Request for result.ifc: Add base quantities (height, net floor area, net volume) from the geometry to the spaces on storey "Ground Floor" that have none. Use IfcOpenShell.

First a look at what the model holds.

```python
import ifcopenshell
import ifcopenshell.util.element
import ifcopenshell.util.unit

model = ifcopenshell.open("result.ifc")
print(model.schema)
for unit_type in ("LENGTHUNIT", "AREAUNIT", "VOLUMEUNIT"):
    print(unit_type, ifcopenshell.util.unit.calculate_unit_scale(model, unit_type))
storey = next(s for s in model.by_type("IfcBuildingStorey") if s.Name == "Ground Floor")
spaces = [e for e in ifcopenshell.util.element.get_decomposition(storey) if e.is_a("IfcSpace")]
for e in sorted(spaces, key=lambda e: e.id()):
    print(e.id(), e.is_a(), e.Name, list(ifcopenshell.util.element.get_psets(e, qtos_only=True)), sep=" | ")
```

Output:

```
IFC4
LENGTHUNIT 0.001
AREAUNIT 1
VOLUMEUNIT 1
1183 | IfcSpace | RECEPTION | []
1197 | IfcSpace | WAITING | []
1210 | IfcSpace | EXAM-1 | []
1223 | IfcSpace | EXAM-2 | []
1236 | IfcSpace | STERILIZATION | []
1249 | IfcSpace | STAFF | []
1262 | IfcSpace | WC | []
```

```python
import ifcopenshell
import ifcopenshell.api.pset
import ifcopenshell.geom
import ifcopenshell.util.element
import ifcopenshell.util.shape
import ifcopenshell.util.unit

model = ifcopenshell.open("result.ifc")
unit_scale = ifcopenshell.util.unit.calculate_unit_scale(model)
area_scale = ifcopenshell.util.unit.calculate_unit_scale(model, "AREAUNIT")
volume_scale = ifcopenshell.util.unit.calculate_unit_scale(model, "VOLUMEUNIT")
settings = ifcopenshell.geom.settings()

storey = next(s for s in model.by_type("IfcBuildingStorey") if s.Name == "Ground Floor")
spaces = [e for e in ifcopenshell.util.element.get_decomposition(storey) if e.is_a("IfcSpace")]

for e in sorted(spaces, key=lambda e: e.id()):
    if ifcopenshell.util.element.get_psets(e, qtos_only=True, should_inherit=False):
        continue
    # Geometry comes back in metres, in the element's own axes.
    shape = ifcopenshell.geom.create_shape(settings, e)
    values = {
        "Height": ifcopenshell.util.shape.get_z(shape.geometry) / unit_scale,
        "NetFloorArea": ifcopenshell.util.shape.get_footprint_area(shape.geometry) / area_scale,
        "NetVolume": ifcopenshell.util.shape.get_volume(shape.geometry) / volume_scale,
    }
    qto = ifcopenshell.api.pset.add_qto(model, product=e, name="Qto_SpaceBaseQuantities")
    ifcopenshell.api.pset.edit_qto(model, qto=qto, properties=values)
    print(e.id(), {k: round(v, 3) for k, v in values.items()})

model.write("result-out.ifc")
```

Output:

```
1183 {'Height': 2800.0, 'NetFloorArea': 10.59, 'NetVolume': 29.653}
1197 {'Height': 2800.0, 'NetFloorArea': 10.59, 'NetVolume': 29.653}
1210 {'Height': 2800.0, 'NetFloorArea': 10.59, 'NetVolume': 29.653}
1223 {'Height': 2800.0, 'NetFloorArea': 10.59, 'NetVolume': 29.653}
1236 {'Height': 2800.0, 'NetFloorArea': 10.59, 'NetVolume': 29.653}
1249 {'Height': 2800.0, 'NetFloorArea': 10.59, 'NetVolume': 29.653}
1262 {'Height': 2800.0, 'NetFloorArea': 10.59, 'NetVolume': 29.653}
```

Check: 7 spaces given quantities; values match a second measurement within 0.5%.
